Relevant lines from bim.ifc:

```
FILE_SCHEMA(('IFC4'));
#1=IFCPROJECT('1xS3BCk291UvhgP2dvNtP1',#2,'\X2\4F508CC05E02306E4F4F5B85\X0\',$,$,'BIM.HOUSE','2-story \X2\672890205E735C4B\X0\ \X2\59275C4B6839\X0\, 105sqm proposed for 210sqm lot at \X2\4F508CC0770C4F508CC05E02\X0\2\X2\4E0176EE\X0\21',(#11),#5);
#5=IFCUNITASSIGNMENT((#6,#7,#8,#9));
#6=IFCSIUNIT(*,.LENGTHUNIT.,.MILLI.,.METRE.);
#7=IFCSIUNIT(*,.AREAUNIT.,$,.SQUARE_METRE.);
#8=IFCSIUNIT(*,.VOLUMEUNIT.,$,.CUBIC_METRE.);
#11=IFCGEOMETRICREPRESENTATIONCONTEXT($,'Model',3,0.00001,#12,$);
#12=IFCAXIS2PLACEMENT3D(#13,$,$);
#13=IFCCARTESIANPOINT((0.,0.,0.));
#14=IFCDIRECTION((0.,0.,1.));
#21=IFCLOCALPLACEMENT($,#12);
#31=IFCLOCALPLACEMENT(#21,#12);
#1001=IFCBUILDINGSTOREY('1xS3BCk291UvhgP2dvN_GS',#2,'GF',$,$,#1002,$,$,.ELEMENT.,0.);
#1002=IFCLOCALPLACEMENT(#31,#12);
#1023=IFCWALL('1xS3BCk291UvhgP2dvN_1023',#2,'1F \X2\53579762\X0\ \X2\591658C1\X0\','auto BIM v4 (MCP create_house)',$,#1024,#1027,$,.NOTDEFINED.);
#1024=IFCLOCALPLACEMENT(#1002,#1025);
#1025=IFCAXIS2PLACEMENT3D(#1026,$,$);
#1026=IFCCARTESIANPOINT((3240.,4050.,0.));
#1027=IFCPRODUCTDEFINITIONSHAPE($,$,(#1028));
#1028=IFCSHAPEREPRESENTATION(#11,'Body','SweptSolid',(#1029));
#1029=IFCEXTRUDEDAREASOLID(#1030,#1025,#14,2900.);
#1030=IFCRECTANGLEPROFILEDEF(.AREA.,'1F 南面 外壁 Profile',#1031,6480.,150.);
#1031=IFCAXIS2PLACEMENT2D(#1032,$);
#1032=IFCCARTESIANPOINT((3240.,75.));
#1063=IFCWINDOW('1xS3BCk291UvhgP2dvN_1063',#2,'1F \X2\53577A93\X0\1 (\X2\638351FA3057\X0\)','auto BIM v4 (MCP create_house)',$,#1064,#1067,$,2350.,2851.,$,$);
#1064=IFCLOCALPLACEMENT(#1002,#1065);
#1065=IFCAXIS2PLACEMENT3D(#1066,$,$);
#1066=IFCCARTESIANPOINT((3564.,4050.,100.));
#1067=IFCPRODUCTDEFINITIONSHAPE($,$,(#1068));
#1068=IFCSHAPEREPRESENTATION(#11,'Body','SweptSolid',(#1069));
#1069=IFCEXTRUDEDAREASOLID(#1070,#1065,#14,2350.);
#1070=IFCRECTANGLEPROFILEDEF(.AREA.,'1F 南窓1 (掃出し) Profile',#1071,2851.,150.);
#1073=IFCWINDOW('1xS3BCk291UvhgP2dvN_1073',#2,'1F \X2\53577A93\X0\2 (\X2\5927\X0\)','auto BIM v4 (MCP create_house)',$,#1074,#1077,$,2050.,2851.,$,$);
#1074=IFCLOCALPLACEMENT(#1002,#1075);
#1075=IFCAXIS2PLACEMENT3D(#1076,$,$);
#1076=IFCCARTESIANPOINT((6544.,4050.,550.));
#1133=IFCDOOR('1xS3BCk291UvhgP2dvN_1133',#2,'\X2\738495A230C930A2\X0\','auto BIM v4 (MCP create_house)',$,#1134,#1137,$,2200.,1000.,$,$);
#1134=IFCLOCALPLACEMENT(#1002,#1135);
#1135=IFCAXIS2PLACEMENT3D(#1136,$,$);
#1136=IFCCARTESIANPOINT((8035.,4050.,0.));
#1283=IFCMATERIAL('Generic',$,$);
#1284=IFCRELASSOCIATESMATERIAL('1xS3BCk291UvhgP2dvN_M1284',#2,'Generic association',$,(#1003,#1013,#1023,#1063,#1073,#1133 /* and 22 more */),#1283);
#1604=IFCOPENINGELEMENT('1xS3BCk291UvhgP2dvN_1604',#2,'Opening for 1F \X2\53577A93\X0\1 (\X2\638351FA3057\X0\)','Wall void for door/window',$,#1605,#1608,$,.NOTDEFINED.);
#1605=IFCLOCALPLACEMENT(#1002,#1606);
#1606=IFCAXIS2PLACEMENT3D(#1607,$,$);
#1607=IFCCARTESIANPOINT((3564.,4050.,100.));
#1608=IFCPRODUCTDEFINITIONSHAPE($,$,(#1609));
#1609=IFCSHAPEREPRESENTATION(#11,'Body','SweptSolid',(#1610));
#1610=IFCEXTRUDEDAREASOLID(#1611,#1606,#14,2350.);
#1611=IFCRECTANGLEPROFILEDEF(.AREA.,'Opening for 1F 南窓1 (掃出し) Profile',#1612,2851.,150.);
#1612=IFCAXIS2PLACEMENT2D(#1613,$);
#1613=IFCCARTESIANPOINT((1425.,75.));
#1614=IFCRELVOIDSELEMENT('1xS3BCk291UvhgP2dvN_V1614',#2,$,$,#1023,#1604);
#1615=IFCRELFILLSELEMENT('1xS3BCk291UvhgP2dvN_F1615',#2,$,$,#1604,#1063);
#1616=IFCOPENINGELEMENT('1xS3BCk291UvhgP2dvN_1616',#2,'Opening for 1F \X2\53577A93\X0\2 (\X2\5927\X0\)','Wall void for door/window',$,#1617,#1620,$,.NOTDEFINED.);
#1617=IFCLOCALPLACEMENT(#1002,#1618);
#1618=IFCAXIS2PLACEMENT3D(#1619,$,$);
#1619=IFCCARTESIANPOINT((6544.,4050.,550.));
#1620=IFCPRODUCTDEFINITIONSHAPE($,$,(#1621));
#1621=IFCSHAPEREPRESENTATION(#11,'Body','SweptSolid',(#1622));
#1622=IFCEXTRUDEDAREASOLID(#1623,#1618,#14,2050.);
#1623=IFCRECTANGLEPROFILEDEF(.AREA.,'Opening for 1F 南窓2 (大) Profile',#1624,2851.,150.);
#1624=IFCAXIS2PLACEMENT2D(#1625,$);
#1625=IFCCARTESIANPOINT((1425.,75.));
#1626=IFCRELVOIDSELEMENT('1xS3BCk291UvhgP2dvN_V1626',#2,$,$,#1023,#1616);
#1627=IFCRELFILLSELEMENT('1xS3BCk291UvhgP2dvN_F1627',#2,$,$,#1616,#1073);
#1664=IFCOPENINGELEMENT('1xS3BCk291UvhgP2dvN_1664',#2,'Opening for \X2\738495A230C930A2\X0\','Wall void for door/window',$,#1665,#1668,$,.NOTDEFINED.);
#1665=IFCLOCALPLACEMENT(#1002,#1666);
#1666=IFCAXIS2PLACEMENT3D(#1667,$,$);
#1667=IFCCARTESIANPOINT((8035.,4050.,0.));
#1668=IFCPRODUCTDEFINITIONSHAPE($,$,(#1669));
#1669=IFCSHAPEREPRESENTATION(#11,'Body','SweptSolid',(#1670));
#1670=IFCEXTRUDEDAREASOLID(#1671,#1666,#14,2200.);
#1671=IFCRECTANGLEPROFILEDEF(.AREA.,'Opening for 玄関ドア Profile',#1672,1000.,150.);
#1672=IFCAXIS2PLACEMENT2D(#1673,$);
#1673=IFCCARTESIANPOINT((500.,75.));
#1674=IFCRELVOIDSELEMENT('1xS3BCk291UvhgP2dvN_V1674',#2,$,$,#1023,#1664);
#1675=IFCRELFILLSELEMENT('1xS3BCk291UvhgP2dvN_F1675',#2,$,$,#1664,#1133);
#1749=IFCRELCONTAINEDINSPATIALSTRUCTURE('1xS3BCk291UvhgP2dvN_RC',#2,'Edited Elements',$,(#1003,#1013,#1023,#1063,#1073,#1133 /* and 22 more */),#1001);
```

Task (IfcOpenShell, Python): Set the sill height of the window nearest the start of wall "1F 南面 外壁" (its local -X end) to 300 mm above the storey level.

```python
import numpy as np
import ifcopenshell
import ifcopenshell.api.geometry
import ifcopenshell.geom
import ifcopenshell.util.element
import ifcopenshell.util.placement
import ifcopenshell.util.shape
import ifcopenshell.util.unit

model = ifcopenshell.open("bim.ifc")
unit_scale = ifcopenshell.util.unit.calculate_unit_scale(model)

window = model.by_guid("1xS3BCk291UvhgP2dvN_1063")
opening = window.FillsVoids[0].RelatingOpeningElement
storey = ifcopenshell.util.element.get_container(window, ifc_class="IfcBuildingStorey")
level = ifcopenshell.util.placement.get_local_placement(storey.ObjectPlacement)[2, 3]

# The opening's origin need not be at the sill, so measure its lowest point.
shape = ifcopenshell.geom.create_shape(ifcopenshell.geom.settings(), opening)
bottom = ifcopenshell.util.shape.get_shape_bottom_elevation(shape, shape.geometry) / unit_scale
dz = level + 0.3 / unit_scale - bottom

shift = np.array([0.0, 0.0, dz])
# The window is not placed relative to its opening, so move both.
for product in (opening, window):
    matrix = ifcopenshell.util.placement.get_local_placement(product.ObjectPlacement)
    matrix[:3, 3] += shift
    ifcopenshell.api.geometry.edit_object_placement(model, product=product, matrix=matrix, is_si=False)

print(f"moved by {dz * unit_scale:+.3f} m")

model.write("bim_rev.ifc")
```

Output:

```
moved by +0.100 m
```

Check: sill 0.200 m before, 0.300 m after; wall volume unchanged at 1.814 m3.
